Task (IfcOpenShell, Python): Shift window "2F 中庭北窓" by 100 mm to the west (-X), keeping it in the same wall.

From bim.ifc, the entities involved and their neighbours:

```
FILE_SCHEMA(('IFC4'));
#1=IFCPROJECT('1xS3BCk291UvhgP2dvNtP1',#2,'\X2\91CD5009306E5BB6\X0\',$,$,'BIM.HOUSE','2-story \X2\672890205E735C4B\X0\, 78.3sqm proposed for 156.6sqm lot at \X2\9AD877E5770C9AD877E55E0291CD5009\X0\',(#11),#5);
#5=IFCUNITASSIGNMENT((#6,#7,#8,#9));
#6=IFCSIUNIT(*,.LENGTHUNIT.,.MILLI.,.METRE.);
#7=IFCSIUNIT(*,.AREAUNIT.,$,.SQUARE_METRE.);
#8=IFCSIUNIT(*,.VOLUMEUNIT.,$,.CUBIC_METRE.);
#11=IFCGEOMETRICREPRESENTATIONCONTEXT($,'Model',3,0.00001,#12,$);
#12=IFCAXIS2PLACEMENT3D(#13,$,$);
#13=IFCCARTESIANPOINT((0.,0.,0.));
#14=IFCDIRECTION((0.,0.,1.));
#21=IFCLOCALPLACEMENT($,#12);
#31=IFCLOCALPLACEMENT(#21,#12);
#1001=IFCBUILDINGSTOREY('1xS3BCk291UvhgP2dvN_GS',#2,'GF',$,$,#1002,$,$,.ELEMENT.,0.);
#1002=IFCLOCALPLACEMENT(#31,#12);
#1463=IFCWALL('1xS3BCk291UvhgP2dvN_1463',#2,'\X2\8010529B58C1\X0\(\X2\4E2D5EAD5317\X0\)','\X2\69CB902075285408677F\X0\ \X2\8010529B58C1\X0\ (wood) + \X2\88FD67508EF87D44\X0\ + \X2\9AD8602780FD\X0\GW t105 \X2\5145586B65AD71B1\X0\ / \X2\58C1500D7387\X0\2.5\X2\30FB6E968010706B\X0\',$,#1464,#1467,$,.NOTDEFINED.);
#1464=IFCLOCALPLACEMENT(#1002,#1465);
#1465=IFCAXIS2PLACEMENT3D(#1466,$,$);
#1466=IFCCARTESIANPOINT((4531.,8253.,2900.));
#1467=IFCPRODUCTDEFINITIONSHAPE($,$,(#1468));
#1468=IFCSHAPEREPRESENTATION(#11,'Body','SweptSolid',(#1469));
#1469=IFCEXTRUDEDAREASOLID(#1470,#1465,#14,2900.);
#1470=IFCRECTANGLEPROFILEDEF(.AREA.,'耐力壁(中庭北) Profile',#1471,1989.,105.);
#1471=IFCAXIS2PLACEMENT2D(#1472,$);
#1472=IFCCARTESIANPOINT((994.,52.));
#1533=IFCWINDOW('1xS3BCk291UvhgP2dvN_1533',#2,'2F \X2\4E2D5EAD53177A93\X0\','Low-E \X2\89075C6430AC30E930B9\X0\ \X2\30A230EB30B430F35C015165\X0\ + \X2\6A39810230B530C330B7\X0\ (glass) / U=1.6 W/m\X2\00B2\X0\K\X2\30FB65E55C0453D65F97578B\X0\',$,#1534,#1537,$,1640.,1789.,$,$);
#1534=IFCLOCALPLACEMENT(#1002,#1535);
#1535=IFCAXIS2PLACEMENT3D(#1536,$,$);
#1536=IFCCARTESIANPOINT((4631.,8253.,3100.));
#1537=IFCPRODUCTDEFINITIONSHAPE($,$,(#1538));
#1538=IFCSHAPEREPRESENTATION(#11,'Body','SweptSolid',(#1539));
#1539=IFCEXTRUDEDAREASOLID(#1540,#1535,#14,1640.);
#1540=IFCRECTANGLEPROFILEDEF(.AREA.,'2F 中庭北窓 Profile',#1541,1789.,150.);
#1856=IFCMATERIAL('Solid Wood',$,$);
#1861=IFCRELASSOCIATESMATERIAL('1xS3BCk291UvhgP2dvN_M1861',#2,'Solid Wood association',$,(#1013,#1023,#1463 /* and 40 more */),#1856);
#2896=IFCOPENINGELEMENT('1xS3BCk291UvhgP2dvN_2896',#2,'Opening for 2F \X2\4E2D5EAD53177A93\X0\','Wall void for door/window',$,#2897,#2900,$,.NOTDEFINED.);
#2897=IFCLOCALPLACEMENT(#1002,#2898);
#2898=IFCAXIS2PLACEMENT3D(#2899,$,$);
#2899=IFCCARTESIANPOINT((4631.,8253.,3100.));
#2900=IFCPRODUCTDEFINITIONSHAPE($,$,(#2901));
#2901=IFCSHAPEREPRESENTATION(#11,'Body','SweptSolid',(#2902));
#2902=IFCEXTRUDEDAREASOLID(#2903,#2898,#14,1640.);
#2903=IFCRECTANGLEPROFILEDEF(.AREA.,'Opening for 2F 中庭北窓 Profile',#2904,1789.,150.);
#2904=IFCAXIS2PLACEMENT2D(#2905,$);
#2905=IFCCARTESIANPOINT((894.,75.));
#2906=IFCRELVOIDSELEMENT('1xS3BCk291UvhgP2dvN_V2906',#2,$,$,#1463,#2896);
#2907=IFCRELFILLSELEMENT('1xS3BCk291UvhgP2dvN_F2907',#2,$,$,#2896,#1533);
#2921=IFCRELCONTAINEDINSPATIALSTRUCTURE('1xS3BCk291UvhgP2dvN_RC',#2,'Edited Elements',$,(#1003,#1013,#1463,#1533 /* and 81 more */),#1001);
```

```python
import ifcopenshell
import ifcopenshell.api.geometry
import ifcopenshell.util.placement
import ifcopenshell.util.unit

model = ifcopenshell.open("bim.ifc")
unit_scale = ifcopenshell.util.unit.calculate_unit_scale(model)

window = model.by_guid("1xS3BCk291UvhgP2dvN_1533")
opening = window.FillsVoids[0].RelatingOpeningElement
wall = opening.VoidsElements[0].RelatingBuildingElement

wall_matrix = ifcopenshell.util.placement.get_local_placement(wall.ObjectPlacement)
shift = wall_matrix[:3, 0] * -0.1 / unit_scale
before = ifcopenshell.util.placement.get_local_placement(window.ObjectPlacement)[:3, 3].copy()

# The window is not placed relative to its opening, so move both.
for product in (opening, window):
    matrix = ifcopenshell.util.placement.get_local_placement(product.ObjectPlacement)
    matrix[:3, 3] += shift
    ifcopenshell.api.geometry.edit_object_placement(model, product=product, matrix=matrix, is_si=False)

after = ifcopenshell.util.placement.get_local_placement(window.ObjectPlacement)[:3, 3]
print("window moved by", (after - before).round(3) + 0.0)

model.write("bim-out.ifc")
```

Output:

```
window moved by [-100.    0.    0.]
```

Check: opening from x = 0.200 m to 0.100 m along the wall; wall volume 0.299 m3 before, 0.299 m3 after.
